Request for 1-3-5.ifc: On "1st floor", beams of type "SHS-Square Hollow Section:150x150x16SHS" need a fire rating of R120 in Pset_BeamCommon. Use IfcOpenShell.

First a look at what the model holds.

```python
import ifcopenshell
import ifcopenshell.util.element

model = ifcopenshell.open("1-3-5.ifc")
print(model.schema)
storey = next(s for s in model.by_type("IfcBuildingStorey") if s.Name == "1st floor")
beams = [e for e in ifcopenshell.util.element.get_decomposition(storey) if e.is_a("IfcBeam")]
seen = {}
for e in beams:
    element_type = ifcopenshell.util.element.get_type(e)
    key = (element_type.Name if element_type != e and element_type else None, ifcopenshell.util.element.get_pset(e, "Pset_BeamCommon", "FireRating"))
    seen[key] = seen.get(key, 0) + 1
for (name, value), count in sorted(seen.items(), key=str):
    print(count, "x", name, "|", value)
```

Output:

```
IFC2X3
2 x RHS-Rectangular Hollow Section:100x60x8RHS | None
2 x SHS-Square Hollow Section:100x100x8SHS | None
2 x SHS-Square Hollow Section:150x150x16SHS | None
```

```python
import ifcopenshell
import ifcopenshell.api.pset
import ifcopenshell.util.element

model = ifcopenshell.open("1-3-5.ifc")

storey = next(s for s in model.by_type("IfcBuildingStorey") if s.Name == "1st floor")
beams = [e for e in ifcopenshell.util.element.get_decomposition(storey) if e.is_a("IfcBeam")]

count = 0
for e in beams:
    element_type = ifcopenshell.util.element.get_type(e)
    if element_type in (None, e) or element_type.Name != "SHS-Square Hollow Section:150x150x16SHS":
        continue
    # add_pset returns the element's existing set when there is one.
    pset = ifcopenshell.api.pset.add_pset(model, product=e, name="Pset_BeamCommon")
    ifcopenshell.api.pset.edit_pset(model, pset=pset, properties={"FireRating": "R120"})
    count += 1

print(count, "beams updated")

model.write("1-3-5-out.ifc")
```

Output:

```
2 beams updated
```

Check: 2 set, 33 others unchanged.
